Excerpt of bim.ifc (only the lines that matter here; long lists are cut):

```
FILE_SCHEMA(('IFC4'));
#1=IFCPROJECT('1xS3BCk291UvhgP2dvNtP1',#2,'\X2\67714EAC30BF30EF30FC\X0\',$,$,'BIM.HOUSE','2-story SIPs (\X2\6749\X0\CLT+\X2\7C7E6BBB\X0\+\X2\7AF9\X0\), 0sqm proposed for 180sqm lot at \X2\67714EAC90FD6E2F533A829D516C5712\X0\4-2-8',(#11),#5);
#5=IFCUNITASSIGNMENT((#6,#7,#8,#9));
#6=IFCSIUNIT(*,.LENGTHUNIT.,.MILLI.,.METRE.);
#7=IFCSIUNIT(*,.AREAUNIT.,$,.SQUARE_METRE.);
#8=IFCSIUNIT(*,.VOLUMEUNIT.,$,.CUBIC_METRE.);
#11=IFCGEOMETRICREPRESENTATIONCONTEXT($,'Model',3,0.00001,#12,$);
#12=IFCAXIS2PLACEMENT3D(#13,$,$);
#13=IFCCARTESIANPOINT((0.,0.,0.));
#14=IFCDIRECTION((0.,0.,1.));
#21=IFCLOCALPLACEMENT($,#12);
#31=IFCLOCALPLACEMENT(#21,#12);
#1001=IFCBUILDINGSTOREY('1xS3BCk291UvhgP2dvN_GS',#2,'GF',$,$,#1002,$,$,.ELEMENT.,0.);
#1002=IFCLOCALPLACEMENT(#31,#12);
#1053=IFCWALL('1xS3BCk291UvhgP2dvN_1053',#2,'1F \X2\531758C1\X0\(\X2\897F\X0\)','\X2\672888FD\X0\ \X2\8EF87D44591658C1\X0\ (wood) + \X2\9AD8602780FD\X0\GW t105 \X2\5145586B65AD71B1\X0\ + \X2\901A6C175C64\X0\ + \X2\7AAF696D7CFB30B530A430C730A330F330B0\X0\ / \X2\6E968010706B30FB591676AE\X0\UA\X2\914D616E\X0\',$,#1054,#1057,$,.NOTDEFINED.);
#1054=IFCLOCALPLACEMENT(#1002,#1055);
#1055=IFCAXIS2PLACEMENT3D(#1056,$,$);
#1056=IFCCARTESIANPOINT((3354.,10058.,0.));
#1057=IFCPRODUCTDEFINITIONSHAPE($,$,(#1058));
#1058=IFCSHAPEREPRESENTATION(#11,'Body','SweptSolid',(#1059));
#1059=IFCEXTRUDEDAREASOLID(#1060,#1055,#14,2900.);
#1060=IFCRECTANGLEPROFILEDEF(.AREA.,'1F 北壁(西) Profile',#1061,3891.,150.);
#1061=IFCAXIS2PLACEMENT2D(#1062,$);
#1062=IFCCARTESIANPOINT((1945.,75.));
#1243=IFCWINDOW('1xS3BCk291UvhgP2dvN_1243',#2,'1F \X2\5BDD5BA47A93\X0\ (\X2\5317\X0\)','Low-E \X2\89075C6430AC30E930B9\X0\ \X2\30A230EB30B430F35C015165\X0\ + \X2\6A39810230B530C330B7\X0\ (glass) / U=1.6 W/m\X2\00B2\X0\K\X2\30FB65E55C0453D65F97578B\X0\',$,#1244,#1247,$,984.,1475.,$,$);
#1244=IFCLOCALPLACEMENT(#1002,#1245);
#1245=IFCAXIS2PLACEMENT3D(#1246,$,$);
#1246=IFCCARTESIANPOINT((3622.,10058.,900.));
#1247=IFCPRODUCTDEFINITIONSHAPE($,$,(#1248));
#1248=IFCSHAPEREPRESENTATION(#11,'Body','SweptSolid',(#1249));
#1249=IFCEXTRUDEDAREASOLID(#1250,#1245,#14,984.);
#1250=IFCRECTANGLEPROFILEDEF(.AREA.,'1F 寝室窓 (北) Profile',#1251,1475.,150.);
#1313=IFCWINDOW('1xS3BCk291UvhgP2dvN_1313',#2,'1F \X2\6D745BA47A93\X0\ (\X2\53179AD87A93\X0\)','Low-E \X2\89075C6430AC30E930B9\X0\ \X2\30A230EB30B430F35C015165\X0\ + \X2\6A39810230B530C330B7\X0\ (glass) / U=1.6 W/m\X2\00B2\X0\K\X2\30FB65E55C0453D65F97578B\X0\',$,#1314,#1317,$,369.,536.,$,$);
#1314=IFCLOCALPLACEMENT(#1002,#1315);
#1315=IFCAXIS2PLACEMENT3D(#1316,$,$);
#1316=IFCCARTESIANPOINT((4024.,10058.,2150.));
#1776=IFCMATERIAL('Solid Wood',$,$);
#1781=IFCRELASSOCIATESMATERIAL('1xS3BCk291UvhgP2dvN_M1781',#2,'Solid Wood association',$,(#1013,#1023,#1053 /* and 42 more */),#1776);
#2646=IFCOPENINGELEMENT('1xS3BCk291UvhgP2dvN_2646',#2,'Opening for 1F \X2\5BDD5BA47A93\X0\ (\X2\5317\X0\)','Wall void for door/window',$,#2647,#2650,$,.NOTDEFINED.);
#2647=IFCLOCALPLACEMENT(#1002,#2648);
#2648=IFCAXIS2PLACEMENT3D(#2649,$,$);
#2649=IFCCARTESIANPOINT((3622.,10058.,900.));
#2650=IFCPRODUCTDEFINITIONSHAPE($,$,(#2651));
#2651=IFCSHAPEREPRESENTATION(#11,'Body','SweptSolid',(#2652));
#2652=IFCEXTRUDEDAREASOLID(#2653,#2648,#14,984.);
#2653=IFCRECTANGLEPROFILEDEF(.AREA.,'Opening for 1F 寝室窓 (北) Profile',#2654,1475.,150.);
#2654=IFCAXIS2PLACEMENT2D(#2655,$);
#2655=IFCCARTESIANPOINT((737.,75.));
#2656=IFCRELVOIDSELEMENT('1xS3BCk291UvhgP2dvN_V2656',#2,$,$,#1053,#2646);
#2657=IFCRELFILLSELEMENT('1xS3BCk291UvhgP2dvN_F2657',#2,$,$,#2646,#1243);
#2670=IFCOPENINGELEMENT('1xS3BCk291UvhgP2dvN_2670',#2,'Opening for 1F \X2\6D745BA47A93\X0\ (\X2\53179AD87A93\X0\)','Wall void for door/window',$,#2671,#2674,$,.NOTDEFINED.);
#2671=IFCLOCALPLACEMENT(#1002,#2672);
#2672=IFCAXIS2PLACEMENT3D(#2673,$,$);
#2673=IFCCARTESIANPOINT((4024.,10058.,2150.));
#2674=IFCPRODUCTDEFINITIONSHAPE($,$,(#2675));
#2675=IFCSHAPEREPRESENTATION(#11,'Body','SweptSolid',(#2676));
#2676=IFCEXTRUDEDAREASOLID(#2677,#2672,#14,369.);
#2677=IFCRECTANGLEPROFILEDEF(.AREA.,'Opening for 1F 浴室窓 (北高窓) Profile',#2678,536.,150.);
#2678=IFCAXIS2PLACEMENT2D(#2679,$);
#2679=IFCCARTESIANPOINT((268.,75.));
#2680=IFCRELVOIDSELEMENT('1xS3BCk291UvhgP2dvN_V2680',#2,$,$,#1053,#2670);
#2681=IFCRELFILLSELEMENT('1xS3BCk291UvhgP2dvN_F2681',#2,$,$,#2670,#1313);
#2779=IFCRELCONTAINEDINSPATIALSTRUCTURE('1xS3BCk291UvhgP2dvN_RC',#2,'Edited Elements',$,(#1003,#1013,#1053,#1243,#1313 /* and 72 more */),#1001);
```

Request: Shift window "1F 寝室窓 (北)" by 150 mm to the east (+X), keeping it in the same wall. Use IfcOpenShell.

```python
import ifcopenshell
import ifcopenshell.api.geometry
import ifcopenshell.util.placement

model = ifcopenshell.open("bim.ifc")

window = model.by_id(1243)
opening = window.FillsVoids[0].RelatingOpeningElement
wall = opening.VoidsElements[0].RelatingBuildingElement

wall_matrix = ifcopenshell.util.placement.get_local_placement(wall.ObjectPlacement)
shift = wall_matrix[:3, 0] * 150.0
before = ifcopenshell.util.placement.get_local_placement(window.ObjectPlacement)[:3, 3].copy()

# The window is not placed relative to its opening, so move both.
for product in (opening, window):
    matrix = ifcopenshell.util.placement.get_local_placement(product.ObjectPlacement)
    matrix[:3, 3] += shift
    ifcopenshell.api.geometry.edit_object_placement(model, product=product, matrix=matrix, is_si=False)

after = ifcopenshell.util.placement.get_local_placement(window.ObjectPlacement)[:3, 3]
print("window moved by", (after - before).round(3) + 0.0)

model.write("bim-out.ifc")
```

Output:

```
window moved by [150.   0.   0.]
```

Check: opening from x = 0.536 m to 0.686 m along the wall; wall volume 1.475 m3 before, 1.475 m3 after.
